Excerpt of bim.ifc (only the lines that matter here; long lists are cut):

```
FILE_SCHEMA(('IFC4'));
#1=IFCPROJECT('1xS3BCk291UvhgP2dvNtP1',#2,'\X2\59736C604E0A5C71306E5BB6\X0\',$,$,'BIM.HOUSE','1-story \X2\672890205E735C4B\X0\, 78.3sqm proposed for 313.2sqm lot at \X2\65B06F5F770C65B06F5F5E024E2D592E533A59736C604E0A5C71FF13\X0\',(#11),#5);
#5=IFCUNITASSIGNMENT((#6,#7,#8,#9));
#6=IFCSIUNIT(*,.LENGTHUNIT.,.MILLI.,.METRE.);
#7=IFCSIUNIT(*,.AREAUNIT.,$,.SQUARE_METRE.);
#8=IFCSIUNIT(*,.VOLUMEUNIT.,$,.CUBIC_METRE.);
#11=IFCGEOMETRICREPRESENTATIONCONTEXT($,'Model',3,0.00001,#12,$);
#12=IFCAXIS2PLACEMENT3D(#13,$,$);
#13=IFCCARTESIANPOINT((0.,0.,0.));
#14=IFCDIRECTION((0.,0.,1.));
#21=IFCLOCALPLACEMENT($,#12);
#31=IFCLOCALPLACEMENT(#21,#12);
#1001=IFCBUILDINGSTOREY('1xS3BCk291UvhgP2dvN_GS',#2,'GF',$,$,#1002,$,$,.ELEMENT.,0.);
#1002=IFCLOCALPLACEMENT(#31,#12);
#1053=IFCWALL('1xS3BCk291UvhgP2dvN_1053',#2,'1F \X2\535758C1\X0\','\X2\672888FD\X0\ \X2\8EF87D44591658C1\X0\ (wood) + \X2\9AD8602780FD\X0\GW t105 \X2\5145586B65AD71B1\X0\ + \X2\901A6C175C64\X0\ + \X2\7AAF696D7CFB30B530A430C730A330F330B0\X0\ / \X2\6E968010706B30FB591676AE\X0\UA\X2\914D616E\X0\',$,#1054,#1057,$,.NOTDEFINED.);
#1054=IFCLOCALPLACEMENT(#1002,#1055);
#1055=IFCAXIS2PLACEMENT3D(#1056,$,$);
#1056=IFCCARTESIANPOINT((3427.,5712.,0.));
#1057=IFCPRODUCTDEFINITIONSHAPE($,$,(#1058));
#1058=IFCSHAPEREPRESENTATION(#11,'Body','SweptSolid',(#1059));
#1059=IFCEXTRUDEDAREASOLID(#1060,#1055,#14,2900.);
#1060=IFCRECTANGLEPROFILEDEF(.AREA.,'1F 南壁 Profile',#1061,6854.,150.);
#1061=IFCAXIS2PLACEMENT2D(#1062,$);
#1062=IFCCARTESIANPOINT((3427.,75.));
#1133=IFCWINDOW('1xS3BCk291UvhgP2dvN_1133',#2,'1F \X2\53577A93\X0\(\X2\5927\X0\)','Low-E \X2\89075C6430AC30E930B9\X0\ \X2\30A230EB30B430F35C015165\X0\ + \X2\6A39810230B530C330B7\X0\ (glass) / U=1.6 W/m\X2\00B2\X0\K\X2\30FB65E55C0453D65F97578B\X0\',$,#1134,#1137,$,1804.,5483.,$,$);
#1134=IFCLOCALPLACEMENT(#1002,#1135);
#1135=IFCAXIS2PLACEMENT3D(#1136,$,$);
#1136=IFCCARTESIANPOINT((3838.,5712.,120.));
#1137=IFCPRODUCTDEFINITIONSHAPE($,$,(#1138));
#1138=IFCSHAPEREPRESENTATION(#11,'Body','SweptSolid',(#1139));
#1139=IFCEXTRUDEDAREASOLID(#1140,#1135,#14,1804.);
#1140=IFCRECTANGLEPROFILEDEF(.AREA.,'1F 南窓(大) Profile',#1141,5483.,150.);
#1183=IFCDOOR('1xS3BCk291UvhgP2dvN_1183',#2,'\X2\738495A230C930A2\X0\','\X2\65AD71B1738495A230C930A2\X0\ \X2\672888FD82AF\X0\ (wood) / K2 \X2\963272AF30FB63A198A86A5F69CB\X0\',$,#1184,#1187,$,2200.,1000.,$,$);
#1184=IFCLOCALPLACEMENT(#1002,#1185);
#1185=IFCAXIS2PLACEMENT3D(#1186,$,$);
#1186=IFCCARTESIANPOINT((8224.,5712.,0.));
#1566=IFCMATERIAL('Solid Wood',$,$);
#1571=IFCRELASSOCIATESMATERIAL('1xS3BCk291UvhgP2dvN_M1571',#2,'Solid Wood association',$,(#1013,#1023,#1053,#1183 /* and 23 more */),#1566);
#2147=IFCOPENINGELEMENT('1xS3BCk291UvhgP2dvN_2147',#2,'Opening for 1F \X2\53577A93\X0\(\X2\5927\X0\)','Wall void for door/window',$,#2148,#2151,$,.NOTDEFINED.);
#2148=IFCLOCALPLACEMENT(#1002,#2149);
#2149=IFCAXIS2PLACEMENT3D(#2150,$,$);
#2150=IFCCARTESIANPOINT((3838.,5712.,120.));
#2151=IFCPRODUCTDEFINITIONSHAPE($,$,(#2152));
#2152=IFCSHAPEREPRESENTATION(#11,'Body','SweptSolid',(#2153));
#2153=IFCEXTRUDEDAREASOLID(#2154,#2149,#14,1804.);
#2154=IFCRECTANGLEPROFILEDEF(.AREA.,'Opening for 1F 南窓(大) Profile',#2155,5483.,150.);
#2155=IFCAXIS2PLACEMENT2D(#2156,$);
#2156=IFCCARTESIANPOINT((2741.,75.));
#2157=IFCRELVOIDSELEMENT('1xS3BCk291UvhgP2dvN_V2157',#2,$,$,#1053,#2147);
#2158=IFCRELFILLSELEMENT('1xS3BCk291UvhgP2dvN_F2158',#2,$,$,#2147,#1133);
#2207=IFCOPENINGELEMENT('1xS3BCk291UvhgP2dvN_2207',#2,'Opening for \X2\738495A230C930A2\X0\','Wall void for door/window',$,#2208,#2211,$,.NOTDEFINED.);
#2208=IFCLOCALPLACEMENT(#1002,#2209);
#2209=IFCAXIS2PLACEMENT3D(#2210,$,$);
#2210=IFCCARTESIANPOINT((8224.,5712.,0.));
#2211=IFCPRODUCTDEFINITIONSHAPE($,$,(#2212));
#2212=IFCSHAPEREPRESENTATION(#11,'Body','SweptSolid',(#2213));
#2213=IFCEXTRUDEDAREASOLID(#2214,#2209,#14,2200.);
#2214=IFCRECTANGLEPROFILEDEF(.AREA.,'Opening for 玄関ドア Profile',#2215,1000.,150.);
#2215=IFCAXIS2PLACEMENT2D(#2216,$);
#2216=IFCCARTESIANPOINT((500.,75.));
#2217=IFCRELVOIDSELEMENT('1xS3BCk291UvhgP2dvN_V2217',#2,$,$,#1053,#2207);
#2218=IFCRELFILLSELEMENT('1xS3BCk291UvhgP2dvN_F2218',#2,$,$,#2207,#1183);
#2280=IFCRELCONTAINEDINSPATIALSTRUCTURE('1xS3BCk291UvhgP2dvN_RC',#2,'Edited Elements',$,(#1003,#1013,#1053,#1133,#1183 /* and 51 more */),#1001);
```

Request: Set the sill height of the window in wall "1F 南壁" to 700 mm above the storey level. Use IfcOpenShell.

```python
import numpy as np
import ifcopenshell
import ifcopenshell.api.geometry
import ifcopenshell.geom
import ifcopenshell.util.element
import ifcopenshell.util.placement
import ifcopenshell.util.shape
import ifcopenshell.util.unit

model = ifcopenshell.open("bim.ifc")
unit_scale = ifcopenshell.util.unit.calculate_unit_scale(model)

window = model.by_guid("1xS3BCk291UvhgP2dvN_1133")
opening = window.FillsVoids[0].RelatingOpeningElement
storey = ifcopenshell.util.element.get_container(window, ifc_class="IfcBuildingStorey")
level = ifcopenshell.util.placement.get_local_placement(storey.ObjectPlacement)[2, 3]

# The opening's origin need not be at the sill, so measure its lowest point.
shape = ifcopenshell.geom.create_shape(ifcopenshell.geom.settings(), opening)
bottom = ifcopenshell.util.shape.get_shape_bottom_elevation(shape, shape.geometry) / unit_scale
dz = level + 0.7 / unit_scale - bottom

shift = np.array([0.0, 0.0, dz])
# The window is not placed relative to its opening, so move both.
for product in (opening, window):
    matrix = ifcopenshell.util.placement.get_local_placement(product.ObjectPlacement)
    matrix[:3, 3] += shift
    ifcopenshell.api.geometry.edit_object_placement(model, product=product, matrix=matrix, is_si=False)

print(f"moved by {dz * unit_scale:+.3f} m")

model.write("bim_rev.ifc")
```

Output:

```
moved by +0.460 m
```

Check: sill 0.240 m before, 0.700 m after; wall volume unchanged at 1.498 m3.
